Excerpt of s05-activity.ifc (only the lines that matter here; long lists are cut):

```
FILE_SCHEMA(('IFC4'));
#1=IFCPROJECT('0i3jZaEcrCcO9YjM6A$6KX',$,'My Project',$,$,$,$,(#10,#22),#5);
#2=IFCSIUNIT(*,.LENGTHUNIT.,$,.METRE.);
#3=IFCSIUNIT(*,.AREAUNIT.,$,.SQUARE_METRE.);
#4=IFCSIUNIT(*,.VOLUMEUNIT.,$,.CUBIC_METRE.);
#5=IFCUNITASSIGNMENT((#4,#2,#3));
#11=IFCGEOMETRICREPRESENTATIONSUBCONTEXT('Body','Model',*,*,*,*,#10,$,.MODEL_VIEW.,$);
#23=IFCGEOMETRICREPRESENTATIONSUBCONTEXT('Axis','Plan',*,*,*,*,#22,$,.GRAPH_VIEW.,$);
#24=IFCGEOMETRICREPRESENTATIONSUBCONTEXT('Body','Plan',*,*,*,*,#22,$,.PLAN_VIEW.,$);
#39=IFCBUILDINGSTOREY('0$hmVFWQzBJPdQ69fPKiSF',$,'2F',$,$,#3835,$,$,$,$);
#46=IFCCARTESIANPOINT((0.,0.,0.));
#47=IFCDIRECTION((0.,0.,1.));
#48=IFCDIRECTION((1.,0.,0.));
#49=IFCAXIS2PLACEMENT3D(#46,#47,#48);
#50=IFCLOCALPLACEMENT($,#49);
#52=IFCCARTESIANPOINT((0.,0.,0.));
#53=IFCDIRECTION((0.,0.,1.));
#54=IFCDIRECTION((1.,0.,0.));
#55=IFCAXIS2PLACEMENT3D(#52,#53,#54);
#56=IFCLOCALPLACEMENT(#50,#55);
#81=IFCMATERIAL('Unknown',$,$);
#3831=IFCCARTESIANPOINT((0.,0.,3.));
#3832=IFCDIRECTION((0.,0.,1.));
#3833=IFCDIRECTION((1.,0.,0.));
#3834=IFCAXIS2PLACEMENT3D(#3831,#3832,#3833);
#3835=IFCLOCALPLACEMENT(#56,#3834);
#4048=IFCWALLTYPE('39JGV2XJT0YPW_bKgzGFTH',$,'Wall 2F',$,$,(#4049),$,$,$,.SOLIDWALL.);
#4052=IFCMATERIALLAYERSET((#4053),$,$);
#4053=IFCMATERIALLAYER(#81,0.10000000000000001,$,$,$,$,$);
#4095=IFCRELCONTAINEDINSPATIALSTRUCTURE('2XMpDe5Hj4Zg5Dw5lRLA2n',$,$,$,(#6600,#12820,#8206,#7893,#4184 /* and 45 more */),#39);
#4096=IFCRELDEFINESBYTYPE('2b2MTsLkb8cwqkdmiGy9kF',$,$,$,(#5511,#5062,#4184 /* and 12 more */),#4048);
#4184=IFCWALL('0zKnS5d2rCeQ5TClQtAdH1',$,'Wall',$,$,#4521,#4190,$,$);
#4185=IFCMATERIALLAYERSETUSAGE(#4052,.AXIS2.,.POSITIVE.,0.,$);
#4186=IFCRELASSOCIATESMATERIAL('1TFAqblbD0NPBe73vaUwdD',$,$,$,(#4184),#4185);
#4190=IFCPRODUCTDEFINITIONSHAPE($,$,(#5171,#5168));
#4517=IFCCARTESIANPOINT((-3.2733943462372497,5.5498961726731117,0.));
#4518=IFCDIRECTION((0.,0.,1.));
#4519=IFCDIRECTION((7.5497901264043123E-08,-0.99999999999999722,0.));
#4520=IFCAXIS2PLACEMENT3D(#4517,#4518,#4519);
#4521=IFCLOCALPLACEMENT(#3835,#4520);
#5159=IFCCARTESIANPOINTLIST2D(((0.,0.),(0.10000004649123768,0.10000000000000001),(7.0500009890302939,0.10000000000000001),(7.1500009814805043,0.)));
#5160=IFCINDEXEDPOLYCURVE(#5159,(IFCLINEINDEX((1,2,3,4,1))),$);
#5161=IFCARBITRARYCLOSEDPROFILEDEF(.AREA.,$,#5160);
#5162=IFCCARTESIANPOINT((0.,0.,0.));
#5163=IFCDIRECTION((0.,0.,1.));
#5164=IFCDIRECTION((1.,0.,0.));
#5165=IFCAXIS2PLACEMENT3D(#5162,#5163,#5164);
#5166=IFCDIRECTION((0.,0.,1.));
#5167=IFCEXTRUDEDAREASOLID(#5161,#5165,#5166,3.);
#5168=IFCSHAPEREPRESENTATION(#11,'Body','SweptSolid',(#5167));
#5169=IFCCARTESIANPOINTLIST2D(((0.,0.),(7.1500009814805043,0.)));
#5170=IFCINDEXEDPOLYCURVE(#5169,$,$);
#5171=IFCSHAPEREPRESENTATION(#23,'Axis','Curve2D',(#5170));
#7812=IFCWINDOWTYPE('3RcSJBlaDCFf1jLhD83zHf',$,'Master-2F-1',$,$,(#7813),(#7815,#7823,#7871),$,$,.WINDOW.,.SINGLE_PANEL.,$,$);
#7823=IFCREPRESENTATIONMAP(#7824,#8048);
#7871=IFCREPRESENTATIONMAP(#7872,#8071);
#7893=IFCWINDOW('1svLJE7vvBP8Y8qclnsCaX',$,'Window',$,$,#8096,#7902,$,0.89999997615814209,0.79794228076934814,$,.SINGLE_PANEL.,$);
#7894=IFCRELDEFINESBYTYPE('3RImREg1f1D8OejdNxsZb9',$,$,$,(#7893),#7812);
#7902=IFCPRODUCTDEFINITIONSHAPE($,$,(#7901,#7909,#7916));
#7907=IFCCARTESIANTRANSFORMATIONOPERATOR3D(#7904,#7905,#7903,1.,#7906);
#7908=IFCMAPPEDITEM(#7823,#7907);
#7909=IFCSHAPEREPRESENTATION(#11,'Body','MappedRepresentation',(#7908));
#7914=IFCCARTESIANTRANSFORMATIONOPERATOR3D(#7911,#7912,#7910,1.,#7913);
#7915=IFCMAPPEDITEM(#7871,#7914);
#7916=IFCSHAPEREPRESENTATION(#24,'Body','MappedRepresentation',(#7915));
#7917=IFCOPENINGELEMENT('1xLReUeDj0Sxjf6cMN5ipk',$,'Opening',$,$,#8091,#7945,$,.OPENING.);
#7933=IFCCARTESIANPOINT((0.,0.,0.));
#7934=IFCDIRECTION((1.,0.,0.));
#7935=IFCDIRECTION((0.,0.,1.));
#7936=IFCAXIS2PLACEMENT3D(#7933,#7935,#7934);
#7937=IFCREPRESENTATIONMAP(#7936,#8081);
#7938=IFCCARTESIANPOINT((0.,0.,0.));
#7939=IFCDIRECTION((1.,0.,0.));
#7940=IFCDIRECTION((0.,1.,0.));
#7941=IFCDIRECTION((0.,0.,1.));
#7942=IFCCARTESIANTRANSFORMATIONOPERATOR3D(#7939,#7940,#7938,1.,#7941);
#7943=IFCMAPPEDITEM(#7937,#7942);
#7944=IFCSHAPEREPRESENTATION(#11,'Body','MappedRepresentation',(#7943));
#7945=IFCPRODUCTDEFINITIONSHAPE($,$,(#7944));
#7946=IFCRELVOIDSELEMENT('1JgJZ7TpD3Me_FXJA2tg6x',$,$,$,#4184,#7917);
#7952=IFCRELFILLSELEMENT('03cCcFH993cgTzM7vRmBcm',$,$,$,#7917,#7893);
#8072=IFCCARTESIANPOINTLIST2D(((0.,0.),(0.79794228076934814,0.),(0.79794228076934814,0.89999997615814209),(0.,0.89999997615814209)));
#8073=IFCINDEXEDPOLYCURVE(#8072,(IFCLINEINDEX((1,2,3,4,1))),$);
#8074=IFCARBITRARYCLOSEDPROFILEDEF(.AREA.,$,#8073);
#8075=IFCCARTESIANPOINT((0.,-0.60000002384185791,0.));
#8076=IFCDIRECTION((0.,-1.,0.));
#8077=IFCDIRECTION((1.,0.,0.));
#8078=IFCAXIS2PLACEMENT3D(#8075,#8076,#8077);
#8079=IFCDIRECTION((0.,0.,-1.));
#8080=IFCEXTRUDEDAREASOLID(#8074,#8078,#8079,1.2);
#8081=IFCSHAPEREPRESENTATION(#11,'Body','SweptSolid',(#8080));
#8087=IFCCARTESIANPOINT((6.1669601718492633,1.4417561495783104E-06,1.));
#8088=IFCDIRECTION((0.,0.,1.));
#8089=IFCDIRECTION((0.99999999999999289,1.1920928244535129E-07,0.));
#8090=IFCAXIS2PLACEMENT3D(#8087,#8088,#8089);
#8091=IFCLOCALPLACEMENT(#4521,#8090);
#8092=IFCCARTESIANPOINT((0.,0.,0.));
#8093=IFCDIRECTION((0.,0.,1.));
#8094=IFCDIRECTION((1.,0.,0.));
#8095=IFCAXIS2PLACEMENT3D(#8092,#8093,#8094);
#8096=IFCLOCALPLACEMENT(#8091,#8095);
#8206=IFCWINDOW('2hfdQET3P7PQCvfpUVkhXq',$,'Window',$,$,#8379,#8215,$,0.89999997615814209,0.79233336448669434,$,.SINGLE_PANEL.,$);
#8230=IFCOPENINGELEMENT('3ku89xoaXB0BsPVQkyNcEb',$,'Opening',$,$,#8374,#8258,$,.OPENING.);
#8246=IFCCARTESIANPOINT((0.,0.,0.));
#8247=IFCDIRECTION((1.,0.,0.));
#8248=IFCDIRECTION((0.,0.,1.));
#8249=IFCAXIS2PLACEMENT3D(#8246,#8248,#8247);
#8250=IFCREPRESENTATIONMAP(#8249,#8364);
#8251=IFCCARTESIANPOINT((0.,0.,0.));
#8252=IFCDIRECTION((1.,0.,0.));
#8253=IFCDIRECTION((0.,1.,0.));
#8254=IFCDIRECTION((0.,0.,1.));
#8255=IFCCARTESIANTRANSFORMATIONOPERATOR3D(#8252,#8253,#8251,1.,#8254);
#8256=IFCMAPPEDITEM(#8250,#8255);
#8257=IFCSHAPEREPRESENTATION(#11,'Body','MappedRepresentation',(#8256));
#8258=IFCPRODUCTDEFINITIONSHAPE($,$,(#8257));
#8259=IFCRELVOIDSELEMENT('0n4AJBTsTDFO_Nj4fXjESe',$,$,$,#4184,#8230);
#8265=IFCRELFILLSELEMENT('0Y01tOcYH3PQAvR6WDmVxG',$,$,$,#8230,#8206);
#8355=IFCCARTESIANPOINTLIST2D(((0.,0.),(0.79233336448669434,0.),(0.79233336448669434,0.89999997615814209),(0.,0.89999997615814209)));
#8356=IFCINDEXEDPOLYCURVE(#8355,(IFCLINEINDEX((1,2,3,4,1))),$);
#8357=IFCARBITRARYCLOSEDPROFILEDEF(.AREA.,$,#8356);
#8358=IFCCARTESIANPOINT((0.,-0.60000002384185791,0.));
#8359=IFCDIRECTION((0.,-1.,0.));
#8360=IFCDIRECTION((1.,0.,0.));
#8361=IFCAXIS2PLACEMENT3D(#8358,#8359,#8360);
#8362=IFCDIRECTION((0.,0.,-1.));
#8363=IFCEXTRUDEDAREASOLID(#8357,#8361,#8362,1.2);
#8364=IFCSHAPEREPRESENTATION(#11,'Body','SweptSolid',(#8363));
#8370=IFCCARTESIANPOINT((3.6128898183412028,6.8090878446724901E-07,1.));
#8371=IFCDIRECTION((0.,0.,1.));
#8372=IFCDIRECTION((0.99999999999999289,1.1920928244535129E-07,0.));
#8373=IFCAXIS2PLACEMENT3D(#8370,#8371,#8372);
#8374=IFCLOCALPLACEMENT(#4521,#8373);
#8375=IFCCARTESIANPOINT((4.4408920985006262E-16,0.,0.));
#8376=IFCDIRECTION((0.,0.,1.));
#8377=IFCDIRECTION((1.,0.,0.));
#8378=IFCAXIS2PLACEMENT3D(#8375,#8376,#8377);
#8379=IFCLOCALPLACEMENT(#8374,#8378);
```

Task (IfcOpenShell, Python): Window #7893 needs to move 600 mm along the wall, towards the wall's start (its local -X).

```python
import ifcopenshell
import ifcopenshell.api.geometry
import ifcopenshell.util.placement
import ifcopenshell.util.unit

model = ifcopenshell.open("s05-activity.ifc")
unit_scale = ifcopenshell.util.unit.calculate_unit_scale(model)

window = model.by_id(7893)
opening = window.FillsVoids[0].RelatingOpeningElement
wall = opening.VoidsElements[0].RelatingBuildingElement

wall_matrix = ifcopenshell.util.placement.get_local_placement(wall.ObjectPlacement)
shift = wall_matrix[:3, 0] * -0.6 / unit_scale
before = ifcopenshell.util.placement.get_local_placement(window.ObjectPlacement)[:3, 3].copy()

# The window is placed relative to its opening, so it follows when the opening moves.
matrix = ifcopenshell.util.placement.get_local_placement(opening.ObjectPlacement)
matrix[:3, 3] += shift
ifcopenshell.api.geometry.edit_object_placement(
    model, product=opening, matrix=matrix, is_si=False, should_transform_children=True
)

after = ifcopenshell.util.placement.get_local_placement(window.ObjectPlacement)[:3, 3]
print("window moved by", (after - before).round(3) + 0.0)

model.write("s05-activity_v2.ifc")
```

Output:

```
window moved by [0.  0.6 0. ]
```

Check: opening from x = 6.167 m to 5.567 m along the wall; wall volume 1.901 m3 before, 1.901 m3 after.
